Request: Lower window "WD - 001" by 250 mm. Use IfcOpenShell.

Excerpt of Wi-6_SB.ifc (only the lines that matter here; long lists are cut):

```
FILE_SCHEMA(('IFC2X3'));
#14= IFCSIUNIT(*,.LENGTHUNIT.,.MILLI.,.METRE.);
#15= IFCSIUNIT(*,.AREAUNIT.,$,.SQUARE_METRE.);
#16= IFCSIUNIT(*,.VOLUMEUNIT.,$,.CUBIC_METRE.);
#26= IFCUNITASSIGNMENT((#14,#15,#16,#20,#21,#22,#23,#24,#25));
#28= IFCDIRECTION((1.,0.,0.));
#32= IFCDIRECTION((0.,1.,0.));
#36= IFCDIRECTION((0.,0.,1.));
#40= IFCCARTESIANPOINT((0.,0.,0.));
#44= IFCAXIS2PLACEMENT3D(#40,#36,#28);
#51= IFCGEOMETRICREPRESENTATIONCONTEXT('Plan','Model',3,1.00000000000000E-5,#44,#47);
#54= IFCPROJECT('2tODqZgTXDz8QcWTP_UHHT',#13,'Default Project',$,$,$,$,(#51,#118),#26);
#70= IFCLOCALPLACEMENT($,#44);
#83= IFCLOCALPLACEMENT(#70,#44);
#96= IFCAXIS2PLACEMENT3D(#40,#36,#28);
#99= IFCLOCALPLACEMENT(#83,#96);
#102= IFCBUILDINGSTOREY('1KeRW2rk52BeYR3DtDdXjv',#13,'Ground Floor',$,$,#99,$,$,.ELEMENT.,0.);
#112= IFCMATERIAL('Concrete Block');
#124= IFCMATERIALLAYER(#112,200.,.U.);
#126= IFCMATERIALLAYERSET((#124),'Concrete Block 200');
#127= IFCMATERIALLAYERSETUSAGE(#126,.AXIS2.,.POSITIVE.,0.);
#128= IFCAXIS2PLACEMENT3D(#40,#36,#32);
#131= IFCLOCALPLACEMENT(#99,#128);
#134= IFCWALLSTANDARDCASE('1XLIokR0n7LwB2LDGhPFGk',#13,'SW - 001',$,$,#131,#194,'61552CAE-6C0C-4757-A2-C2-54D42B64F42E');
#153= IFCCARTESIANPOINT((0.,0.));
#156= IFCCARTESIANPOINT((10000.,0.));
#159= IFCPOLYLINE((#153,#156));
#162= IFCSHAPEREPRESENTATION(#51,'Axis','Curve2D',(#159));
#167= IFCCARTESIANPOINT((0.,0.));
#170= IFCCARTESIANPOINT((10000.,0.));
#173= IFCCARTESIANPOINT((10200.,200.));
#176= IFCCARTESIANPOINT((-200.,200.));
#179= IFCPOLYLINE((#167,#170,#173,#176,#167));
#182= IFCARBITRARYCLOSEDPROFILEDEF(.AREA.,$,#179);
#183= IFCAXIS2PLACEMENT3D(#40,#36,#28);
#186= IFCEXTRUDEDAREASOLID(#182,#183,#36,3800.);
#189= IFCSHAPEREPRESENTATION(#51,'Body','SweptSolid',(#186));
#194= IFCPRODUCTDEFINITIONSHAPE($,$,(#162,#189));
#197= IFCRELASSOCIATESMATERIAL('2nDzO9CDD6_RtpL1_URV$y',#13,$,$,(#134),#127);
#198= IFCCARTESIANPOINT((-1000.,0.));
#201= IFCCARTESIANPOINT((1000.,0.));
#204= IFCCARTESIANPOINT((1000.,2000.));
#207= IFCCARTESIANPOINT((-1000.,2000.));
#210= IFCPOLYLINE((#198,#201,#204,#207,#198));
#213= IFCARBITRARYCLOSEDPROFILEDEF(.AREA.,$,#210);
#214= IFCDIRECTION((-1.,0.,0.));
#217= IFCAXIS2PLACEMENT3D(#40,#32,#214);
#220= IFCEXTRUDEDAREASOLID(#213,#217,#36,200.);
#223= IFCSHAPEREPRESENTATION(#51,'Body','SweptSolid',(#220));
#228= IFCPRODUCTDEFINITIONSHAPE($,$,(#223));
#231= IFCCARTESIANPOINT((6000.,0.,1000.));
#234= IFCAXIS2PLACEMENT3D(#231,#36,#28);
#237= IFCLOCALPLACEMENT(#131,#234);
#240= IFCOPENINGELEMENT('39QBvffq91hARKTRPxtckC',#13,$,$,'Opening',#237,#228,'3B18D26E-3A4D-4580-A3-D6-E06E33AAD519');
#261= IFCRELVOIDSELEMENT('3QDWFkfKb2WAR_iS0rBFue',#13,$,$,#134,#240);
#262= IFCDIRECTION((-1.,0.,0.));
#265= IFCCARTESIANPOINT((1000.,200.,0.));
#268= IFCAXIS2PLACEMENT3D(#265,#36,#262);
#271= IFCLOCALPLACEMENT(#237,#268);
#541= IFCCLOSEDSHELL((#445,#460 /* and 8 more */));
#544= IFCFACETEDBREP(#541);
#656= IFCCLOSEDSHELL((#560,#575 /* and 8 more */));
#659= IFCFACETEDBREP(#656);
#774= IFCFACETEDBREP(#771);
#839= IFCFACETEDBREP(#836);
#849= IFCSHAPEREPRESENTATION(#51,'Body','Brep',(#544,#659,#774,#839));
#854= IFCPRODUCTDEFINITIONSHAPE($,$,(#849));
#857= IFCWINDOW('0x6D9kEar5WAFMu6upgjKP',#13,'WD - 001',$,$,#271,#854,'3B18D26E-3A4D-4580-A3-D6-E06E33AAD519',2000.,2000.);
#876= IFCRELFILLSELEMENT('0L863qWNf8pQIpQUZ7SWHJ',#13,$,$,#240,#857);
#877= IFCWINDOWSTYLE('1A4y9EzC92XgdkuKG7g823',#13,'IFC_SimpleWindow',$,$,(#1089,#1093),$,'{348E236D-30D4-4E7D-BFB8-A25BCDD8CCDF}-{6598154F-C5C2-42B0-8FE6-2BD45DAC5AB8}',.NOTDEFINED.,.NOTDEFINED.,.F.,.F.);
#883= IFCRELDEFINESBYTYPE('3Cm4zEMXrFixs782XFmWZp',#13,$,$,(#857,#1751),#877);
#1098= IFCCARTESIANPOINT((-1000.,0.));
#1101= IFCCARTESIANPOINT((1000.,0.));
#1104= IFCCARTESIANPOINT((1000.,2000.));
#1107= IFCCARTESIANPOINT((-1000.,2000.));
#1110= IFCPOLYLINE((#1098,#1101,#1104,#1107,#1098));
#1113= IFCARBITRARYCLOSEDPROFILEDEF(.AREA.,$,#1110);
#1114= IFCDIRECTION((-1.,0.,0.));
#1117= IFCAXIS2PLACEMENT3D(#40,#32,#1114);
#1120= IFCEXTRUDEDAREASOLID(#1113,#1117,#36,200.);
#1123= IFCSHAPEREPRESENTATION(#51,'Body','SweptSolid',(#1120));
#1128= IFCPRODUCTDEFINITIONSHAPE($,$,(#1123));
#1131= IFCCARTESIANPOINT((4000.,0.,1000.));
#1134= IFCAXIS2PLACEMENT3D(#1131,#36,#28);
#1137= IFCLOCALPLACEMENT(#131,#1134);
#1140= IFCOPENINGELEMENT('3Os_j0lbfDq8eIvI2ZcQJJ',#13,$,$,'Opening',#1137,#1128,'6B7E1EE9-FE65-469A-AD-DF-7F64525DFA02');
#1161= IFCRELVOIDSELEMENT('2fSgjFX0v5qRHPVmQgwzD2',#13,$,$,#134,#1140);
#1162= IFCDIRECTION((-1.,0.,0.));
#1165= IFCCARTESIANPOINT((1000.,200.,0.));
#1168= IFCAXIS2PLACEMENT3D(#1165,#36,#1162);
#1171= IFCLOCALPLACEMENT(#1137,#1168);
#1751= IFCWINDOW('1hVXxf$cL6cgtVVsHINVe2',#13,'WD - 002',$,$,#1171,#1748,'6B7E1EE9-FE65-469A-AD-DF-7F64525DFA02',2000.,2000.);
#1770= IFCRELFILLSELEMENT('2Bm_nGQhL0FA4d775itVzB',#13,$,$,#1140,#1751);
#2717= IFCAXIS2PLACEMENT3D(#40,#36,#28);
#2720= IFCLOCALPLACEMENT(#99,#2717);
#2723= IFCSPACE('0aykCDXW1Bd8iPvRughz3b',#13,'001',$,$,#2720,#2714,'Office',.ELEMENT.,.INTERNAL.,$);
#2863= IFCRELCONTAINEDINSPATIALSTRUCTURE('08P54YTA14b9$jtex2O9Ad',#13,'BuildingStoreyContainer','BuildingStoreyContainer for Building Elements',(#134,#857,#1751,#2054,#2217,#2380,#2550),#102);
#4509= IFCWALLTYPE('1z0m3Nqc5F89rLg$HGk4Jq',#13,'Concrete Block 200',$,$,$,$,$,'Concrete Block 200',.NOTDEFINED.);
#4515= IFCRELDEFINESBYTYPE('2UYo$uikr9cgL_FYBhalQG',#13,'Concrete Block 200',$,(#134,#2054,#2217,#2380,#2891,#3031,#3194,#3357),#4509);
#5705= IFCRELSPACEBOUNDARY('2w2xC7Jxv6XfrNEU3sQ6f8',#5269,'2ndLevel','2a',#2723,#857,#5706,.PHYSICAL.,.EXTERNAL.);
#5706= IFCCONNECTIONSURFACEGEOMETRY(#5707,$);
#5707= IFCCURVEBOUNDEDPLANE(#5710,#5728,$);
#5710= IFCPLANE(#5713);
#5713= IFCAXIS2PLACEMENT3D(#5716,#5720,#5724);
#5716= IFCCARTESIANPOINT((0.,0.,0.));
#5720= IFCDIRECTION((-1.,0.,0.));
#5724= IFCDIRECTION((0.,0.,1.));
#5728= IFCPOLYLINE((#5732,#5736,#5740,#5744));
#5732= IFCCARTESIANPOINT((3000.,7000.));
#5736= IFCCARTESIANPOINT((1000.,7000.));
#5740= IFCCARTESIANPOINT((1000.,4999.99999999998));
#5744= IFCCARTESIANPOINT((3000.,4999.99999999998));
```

```python
import numpy as np
import ifcopenshell
import ifcopenshell.api.geometry
import ifcopenshell.util.placement
import ifcopenshell.util.unit

model = ifcopenshell.open("Wi-6_SB.ifc")
unit_scale = ifcopenshell.util.unit.calculate_unit_scale(model)

window = model.by_guid("0x6D9kEar5WAFMu6upgjKP")
opening = window.FillsVoids[0].RelatingOpeningElement
dz = -250.0

shift = np.array([0.0, 0.0, dz])
# The window is placed relative to its opening, so it follows when the opening moves.
matrix = ifcopenshell.util.placement.get_local_placement(opening.ObjectPlacement)
matrix[:3, 3] += shift
ifcopenshell.api.geometry.edit_object_placement(
    model, product=opening, matrix=matrix, is_si=False, should_transform_children=True
)

# Space boundary surfaces are stored in each space's coordinates; move them too.
for rel in window.ProvidesBoundaries:
    if not rel.ConnectionGeometry:
        continue
    surface = rel.ConnectionGeometry.SurfaceOnRelatingElement.BasisSurface
    space_matrix = ifcopenshell.util.placement.get_local_placement(rel.RelatingSpace.ObjectPlacement)
    point = np.array(surface.Position.Location.Coordinates) + space_matrix[:3, :3].T @ shift
    surface.Position = model.createIfcAxis2Placement3D(
        model.createIfcCartesianPoint(point.tolist()), surface.Position.Axis, surface.Position.RefDirection
    )

print(f"moved by {dz * unit_scale:+.3f} m")

model.write("Wi-6_SB-out.ifc")
```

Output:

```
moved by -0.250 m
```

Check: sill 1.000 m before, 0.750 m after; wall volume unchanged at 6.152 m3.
